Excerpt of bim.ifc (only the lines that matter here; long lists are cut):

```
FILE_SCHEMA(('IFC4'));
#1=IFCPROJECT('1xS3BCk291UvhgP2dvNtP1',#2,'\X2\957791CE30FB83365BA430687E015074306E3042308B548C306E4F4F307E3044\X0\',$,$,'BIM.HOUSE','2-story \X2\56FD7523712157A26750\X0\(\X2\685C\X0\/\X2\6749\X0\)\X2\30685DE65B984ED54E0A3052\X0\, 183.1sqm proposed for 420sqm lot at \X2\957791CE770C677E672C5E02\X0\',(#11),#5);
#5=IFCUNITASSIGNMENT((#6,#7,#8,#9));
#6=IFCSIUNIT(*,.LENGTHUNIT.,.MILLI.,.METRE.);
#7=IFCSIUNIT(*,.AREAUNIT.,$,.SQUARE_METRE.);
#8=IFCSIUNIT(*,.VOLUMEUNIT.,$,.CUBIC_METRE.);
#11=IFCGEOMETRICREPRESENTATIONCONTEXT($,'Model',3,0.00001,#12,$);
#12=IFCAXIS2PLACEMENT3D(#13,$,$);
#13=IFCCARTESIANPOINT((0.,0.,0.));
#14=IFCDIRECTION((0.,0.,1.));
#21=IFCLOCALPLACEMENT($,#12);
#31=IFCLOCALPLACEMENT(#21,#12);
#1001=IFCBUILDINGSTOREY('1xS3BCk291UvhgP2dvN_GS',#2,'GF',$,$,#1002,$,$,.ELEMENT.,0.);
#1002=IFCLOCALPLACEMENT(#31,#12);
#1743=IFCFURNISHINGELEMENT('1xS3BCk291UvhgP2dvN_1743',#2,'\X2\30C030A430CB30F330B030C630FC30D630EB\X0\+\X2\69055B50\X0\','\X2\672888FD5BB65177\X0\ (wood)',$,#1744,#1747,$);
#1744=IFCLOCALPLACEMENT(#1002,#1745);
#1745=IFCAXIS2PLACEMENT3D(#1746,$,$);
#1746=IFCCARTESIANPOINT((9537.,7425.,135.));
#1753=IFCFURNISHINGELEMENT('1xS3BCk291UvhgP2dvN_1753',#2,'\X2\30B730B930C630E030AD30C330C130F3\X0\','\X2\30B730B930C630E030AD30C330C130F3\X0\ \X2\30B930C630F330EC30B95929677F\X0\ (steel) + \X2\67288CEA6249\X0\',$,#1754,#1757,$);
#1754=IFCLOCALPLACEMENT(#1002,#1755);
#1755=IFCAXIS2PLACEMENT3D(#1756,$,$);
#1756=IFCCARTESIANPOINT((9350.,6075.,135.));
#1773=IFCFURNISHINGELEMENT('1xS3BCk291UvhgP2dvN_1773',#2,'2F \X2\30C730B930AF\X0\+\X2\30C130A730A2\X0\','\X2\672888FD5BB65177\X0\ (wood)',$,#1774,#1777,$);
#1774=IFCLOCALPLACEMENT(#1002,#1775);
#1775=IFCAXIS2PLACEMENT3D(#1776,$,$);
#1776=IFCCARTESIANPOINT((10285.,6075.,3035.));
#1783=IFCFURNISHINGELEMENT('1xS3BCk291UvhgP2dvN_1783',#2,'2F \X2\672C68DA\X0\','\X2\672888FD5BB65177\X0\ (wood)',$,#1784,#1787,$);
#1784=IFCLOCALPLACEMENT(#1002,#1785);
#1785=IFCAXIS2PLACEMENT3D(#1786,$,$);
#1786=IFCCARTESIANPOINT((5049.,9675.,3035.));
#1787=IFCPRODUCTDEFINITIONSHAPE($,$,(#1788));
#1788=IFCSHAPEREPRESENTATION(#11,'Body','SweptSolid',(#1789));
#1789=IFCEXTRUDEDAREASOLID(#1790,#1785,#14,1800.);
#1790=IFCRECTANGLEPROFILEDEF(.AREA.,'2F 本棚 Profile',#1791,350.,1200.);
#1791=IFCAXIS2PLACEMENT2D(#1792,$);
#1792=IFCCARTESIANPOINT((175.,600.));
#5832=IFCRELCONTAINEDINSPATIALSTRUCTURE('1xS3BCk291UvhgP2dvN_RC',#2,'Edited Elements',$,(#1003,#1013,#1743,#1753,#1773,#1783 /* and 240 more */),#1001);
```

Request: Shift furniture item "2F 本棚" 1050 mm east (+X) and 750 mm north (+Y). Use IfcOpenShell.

```python
import ifcopenshell
import ifcopenshell.api.geometry
import ifcopenshell.util.placement
import ifcopenshell.util.unit

model = ifcopenshell.open("bim.ifc")
unit_scale = ifcopenshell.util.unit.calculate_unit_scale(model)

item = model.by_id(1783)
matrix = ifcopenshell.util.placement.get_local_placement(item.ObjectPlacement)
matrix[0, 3] += 1.05 / unit_scale
matrix[1, 3] += 0.75 / unit_scale
ifcopenshell.api.geometry.edit_object_placement(model, product=item, matrix=matrix, is_si=False)

print(ifcopenshell.util.placement.get_local_placement(item.ObjectPlacement).round(3) + 0.0)

model.write("bim_v2.ifc")
```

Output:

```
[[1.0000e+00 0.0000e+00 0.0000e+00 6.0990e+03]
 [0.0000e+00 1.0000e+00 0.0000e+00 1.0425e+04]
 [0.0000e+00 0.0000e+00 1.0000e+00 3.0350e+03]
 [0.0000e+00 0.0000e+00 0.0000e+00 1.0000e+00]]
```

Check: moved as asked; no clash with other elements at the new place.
